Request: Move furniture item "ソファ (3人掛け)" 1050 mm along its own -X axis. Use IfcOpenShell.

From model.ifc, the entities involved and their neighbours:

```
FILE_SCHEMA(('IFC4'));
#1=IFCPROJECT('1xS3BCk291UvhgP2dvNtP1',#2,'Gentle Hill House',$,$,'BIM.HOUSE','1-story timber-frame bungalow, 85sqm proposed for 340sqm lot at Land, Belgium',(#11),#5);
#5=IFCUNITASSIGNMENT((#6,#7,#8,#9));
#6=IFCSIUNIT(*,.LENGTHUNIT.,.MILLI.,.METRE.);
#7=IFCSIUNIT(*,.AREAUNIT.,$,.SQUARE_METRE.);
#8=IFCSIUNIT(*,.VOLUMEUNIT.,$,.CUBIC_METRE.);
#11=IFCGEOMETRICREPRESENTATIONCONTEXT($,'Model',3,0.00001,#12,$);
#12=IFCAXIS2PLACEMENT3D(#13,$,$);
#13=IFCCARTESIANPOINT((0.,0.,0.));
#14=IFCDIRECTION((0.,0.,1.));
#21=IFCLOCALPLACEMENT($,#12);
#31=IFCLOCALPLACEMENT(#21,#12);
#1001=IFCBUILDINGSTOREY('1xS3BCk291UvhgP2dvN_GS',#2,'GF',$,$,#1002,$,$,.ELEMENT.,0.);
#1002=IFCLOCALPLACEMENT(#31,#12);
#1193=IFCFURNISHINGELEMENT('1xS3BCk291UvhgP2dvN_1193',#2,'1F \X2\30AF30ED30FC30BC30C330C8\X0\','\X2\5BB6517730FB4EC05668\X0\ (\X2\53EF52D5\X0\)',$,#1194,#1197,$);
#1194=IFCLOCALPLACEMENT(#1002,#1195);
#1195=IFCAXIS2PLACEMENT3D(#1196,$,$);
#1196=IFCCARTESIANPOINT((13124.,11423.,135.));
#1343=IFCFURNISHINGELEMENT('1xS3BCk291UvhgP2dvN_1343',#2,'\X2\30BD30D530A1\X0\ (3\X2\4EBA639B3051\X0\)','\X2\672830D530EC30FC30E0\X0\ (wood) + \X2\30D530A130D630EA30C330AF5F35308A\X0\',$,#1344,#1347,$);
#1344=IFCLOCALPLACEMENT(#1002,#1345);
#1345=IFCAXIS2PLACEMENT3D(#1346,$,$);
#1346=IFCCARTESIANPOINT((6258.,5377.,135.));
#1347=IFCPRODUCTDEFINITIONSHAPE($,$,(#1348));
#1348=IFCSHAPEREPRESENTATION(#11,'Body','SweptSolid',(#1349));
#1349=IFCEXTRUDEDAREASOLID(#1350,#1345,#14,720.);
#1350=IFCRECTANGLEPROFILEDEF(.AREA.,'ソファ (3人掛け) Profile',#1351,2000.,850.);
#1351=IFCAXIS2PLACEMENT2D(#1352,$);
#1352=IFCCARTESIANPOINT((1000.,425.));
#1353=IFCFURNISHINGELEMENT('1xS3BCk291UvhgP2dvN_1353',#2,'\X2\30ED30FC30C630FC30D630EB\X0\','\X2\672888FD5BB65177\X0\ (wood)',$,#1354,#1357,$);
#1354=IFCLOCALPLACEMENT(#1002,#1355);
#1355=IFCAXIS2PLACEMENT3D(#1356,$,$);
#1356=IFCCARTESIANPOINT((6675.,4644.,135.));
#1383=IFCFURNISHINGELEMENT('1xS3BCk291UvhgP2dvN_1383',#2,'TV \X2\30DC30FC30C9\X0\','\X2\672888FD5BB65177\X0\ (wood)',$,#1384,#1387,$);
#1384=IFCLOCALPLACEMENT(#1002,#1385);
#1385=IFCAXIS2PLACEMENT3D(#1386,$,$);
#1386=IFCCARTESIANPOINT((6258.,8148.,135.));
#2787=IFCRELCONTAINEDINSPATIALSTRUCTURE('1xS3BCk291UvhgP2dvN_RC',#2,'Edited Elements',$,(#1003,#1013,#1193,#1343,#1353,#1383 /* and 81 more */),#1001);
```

```python
import ifcopenshell
import ifcopenshell.api.geometry
import ifcopenshell.util.placement
import ifcopenshell.util.unit

model = ifcopenshell.open("model.ifc")
unit_scale = ifcopenshell.util.unit.calculate_unit_scale(model)

item = model.by_guid("1xS3BCk291UvhgP2dvN_1343")
matrix = ifcopenshell.util.placement.get_local_placement(item.ObjectPlacement)
matrix[:3, 3] -= matrix[:3, 0] * 1.05 / unit_scale
ifcopenshell.api.geometry.edit_object_placement(model, product=item, matrix=matrix, is_si=False)

print(ifcopenshell.util.placement.get_local_placement(item.ObjectPlacement).round(3) + 0.0)

model.write("model_v2.ifc")
```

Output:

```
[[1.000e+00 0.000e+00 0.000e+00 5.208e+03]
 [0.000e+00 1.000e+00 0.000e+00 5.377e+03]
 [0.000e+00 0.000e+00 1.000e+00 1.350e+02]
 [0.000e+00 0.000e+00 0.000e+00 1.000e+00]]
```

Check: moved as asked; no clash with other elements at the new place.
